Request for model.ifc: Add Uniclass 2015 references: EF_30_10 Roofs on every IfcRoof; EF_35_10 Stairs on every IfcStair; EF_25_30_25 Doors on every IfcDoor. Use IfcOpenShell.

First a look at what the model holds.

```python
import ifcopenshell

model = ifcopenshell.open("model.ifc")
print(model.schema)
print("classifications:", [c.Name for c in model.by_type("IfcClassification")])
for ifc_class in ("IfcDoor", "IfcRoof", "IfcStair", "IfcWall", "IfcWindow"):
    print(ifc_class, len(model.by_type(ifc_class)))
```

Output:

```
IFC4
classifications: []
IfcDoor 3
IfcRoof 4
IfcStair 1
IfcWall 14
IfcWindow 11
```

```python
import ifcopenshell
import ifcopenshell.api.classification

model = ifcopenshell.open("model.ifc")

system = ifcopenshell.api.classification.add_classification(model, classification="Uniclass 2015")

codes = {
    "IfcRoof": ("EF_30_10", "Roofs"),
    "IfcStair": ("EF_35_10", "Stairs"),
    "IfcDoor": ("EF_25_30_25", "Doors"),
}
for ifc_class, (code, name) in codes.items():
    products = model.by_type(ifc_class)
    ifcopenshell.api.classification.add_reference(
        model, products=products, classification=system, identification=code, name=name
    )
    print(code, len(products))

model.write("model-out.ifc")
```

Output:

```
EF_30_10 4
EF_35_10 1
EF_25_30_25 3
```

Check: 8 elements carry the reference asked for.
